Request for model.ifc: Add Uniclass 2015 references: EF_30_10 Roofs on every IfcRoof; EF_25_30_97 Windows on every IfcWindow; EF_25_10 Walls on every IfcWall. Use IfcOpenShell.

First a look at what the model holds.

```python
import ifcopenshell

model = ifcopenshell.open("model.ifc")
print(model.schema)
print("classifications:", [c.Name for c in model.by_type("IfcClassification")])
for ifc_class in ("IfcDoor", "IfcRoof", "IfcStair", "IfcWall", "IfcWindow"):
    print(ifc_class, len(model.by_type(ifc_class)))
```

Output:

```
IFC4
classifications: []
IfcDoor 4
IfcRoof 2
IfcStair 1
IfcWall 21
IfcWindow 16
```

```python
import ifcopenshell
import ifcopenshell.api.classification

model = ifcopenshell.open("model.ifc")

system = ifcopenshell.api.classification.add_classification(model, classification="Uniclass 2015")

codes = {
    "IfcRoof": ("EF_30_10", "Roofs"),
    "IfcWindow": ("EF_25_30_97", "Windows"),
    "IfcWall": ("EF_25_10", "Walls"),
}
for ifc_class, (code, name) in codes.items():
    products = model.by_type(ifc_class)
    ifcopenshell.api.classification.add_reference(
        model, products=products, classification=system, identification=code, name=name
    )
    print(code, len(products))

model.write("model_v2.ifc")
```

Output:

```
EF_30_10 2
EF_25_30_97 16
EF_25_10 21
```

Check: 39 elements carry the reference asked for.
